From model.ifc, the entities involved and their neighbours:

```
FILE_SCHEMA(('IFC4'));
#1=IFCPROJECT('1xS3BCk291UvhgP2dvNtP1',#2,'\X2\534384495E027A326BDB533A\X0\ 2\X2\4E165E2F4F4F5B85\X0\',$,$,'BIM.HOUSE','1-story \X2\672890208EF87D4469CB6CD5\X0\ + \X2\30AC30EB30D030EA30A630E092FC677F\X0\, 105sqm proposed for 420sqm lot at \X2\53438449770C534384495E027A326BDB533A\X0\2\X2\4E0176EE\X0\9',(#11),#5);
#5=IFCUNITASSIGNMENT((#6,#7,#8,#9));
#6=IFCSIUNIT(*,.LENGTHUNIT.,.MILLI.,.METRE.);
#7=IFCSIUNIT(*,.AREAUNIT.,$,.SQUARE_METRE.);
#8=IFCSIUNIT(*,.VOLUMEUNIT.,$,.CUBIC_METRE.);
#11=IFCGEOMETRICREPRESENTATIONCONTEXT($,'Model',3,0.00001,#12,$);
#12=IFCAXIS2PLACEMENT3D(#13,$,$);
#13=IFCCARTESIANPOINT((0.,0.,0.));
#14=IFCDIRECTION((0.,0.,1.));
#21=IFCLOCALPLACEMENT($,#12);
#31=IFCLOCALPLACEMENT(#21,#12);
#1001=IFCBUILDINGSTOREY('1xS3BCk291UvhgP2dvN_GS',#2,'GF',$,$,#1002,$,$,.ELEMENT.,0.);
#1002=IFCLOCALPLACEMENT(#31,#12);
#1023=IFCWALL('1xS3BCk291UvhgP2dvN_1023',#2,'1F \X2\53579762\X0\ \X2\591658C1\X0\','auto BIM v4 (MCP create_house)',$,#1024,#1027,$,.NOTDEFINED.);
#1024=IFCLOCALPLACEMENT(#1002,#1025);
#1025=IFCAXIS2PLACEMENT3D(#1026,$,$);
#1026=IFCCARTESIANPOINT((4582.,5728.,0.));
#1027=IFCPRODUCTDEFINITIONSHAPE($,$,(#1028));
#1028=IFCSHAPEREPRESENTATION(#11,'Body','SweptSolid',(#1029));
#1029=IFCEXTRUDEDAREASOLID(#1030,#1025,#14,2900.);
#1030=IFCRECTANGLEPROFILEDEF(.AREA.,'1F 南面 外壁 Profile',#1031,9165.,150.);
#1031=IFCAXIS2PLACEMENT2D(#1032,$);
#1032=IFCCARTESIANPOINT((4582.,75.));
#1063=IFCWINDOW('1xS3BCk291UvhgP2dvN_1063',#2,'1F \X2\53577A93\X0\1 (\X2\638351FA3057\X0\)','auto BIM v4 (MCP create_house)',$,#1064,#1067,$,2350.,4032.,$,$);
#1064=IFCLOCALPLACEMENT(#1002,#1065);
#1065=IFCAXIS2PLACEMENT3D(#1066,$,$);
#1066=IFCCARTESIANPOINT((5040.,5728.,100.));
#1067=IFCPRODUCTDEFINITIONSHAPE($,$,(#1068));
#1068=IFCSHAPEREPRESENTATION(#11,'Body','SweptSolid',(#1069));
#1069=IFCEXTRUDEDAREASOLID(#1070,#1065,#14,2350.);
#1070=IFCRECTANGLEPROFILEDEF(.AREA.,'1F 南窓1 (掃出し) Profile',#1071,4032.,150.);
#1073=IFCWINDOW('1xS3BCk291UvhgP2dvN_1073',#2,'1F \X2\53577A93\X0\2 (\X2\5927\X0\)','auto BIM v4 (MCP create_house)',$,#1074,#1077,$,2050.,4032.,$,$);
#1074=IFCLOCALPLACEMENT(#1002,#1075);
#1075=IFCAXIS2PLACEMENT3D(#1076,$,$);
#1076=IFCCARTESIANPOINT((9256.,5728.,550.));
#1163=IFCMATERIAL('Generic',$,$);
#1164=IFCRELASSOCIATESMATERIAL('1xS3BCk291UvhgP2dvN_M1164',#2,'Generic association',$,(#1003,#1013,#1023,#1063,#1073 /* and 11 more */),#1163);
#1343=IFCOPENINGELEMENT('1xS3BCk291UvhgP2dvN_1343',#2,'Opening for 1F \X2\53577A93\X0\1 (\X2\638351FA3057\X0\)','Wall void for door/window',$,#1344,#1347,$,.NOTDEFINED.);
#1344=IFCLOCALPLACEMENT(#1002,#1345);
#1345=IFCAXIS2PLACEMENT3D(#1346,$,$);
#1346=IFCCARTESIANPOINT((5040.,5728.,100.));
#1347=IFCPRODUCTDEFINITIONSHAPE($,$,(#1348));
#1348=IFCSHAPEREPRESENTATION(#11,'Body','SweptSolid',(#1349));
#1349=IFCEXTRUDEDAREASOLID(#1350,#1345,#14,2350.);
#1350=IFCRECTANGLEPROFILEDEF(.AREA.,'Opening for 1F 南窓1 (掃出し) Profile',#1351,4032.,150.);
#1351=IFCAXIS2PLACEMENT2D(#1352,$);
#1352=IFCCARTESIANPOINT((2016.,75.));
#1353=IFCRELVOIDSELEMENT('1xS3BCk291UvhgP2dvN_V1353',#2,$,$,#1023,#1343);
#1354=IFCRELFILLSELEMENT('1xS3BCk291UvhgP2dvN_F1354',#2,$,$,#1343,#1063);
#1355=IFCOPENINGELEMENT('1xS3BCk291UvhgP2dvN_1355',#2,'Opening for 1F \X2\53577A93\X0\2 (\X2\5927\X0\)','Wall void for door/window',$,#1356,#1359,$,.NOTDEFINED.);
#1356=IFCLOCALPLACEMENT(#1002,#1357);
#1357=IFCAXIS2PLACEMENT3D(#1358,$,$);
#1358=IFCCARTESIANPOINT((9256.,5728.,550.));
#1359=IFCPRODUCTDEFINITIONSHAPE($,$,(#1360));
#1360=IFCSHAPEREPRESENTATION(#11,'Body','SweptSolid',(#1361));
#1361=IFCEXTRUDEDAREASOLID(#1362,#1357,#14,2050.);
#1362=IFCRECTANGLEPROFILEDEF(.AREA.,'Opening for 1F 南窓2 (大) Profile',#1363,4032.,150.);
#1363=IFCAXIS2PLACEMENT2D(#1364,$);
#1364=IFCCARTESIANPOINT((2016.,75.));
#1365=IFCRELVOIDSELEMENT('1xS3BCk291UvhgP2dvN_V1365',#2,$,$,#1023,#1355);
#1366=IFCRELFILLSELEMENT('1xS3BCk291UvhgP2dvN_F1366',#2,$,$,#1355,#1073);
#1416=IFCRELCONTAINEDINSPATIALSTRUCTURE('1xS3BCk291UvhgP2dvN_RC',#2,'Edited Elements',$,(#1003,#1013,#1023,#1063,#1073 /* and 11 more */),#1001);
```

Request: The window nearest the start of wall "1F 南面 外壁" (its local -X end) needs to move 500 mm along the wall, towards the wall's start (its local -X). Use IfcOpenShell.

```python
import ifcopenshell
import ifcopenshell.api.geometry
import ifcopenshell.util.placement
import ifcopenshell.util.unit

model = ifcopenshell.open("model.ifc")
unit_scale = ifcopenshell.util.unit.calculate_unit_scale(model)

window = model.by_guid("1xS3BCk291UvhgP2dvN_1063")
opening = window.FillsVoids[0].RelatingOpeningElement
wall = opening.VoidsElements[0].RelatingBuildingElement

wall_matrix = ifcopenshell.util.placement.get_local_placement(wall.ObjectPlacement)
shift = wall_matrix[:3, 0] * -0.5 / unit_scale
before = ifcopenshell.util.placement.get_local_placement(window.ObjectPlacement)[:3, 3].copy()

# The window is not placed relative to its opening, so move both.
for product in (opening, window):
    matrix = ifcopenshell.util.placement.get_local_placement(product.ObjectPlacement)
    matrix[:3, 3] += shift
    ifcopenshell.api.geometry.edit_object_placement(model, product=product, matrix=matrix, is_si=False)

after = ifcopenshell.util.placement.get_local_placement(window.ObjectPlacement)[:3, 3]
print("window moved by", (after - before).round(3) + 0.0)

model.write("model_rev.ifc")
```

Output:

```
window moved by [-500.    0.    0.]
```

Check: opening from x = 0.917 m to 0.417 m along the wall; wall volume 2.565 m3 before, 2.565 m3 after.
